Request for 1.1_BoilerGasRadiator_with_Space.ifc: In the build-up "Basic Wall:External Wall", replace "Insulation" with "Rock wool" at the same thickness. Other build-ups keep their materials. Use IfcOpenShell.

First a look at what the model holds.

```python
import ifcopenshell
import ifcopenshell.util.element

model = ifcopenshell.open("1.1_BoilerGasRadiator_with_Space.ifc")
print(model.schema)
for layer_set in model.by_type("IfcMaterialLayerSet"):
    if layer_set.LayerSetName == "Basic Wall:External Wall":
        for layer in layer_set.MaterialLayers:
            print(layer.id(), layer.Material and layer.Material.Name, layer.LayerThickness, sep=" | ")
        print(len(ifcopenshell.util.element.get_elements_by_material(model, layer_set)), "elements and types use it")
print(sorted(m.Name for m in model.by_type("IfcMaterial") if m.Name)[:60])
```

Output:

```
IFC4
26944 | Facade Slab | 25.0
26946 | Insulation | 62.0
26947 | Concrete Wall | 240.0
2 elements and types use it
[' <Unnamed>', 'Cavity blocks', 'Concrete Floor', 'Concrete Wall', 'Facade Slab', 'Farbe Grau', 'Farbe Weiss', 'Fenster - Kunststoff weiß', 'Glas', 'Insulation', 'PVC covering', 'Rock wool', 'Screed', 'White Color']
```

```python
import ifcopenshell
import ifcopenshell.api.material

model = ifcopenshell.open("1.1_BoilerGasRadiator_with_Space.ifc")

layer_set = next(s for s in model.by_type("IfcMaterialLayerSet") if s.LayerSetName == "Basic Wall:External Wall")
layer = next(l for l in layer_set.MaterialLayers if l.Material and l.Material.Name == "Insulation")
material = next(m for m in model.by_type("IfcMaterial") if m.Name == "Rock wool")

# Point this one layer at the other material; renaming the old one would change it everywhere.
ifcopenshell.api.material.edit_layer(model, layer=layer, attributes={}, material=material)

print([l.Material.Name if l.Material else None for l in layer_set.MaterialLayers])

model.write("1.1_BoilerGasRadiator_with_Space_rev.ifc")
```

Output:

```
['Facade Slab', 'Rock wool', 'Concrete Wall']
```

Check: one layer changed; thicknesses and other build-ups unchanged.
